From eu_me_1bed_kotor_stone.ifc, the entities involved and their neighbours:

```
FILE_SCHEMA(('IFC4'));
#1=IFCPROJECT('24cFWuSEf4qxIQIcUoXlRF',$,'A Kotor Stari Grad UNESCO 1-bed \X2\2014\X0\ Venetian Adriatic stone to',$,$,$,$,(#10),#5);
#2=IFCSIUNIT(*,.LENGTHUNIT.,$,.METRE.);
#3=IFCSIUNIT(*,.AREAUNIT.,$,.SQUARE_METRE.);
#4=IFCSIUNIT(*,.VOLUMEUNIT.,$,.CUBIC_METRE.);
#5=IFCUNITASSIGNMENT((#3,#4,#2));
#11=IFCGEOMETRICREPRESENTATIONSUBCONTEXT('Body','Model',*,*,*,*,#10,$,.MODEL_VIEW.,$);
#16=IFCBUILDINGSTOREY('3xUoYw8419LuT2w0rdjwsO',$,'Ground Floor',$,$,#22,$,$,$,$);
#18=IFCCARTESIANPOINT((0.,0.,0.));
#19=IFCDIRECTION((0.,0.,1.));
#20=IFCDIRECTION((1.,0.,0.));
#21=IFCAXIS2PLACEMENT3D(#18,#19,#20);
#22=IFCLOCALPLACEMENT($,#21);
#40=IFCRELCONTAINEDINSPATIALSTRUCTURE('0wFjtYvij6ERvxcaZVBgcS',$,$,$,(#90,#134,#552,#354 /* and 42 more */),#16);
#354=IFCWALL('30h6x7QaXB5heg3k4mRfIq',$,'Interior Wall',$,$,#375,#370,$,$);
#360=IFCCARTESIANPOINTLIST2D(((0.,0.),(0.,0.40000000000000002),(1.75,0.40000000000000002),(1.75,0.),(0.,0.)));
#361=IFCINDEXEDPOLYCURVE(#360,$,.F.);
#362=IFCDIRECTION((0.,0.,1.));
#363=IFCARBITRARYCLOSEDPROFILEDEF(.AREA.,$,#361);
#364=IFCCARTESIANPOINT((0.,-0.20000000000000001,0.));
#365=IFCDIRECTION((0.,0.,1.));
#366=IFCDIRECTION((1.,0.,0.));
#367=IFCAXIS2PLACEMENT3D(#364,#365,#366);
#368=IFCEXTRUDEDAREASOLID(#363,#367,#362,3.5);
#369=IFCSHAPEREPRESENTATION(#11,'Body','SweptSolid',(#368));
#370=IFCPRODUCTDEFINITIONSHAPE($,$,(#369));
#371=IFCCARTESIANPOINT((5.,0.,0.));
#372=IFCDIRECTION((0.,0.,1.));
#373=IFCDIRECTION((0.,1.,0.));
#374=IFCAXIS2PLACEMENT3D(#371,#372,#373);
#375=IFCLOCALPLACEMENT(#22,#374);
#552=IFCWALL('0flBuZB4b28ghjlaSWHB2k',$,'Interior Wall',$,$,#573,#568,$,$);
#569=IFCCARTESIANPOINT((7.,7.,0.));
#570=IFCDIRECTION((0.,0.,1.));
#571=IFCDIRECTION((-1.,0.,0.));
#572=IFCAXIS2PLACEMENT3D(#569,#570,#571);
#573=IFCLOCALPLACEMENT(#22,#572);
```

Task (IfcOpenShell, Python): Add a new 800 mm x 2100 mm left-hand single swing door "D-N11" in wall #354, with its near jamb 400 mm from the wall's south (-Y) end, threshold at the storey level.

```python
import numpy as np
import ifcopenshell
import ifcopenshell.api.feature
import ifcopenshell.api.geometry
import ifcopenshell.api.root
import ifcopenshell.api.spatial
import ifcopenshell.geom
import ifcopenshell.util.element
import ifcopenshell.util.placement
import ifcopenshell.util.representation
import ifcopenshell.util.shape
import ifcopenshell.util.unit

model = ifcopenshell.open("eu_me_1bed_kotor_stone.ifc")
unit_scale = ifcopenshell.util.unit.calculate_unit_scale(model)
settings = ifcopenshell.geom.settings()


def volume(element):
    """Net volume in cubic metres, openings subtracted."""
    shape = ifcopenshell.geom.create_shape(settings, element)
    return ifcopenshell.util.shape.get_volume(shape.geometry)


wall = model.by_id(354)
storey = ifcopenshell.util.element.get_container(wall, ifc_class="IfcBuildingStorey")
context = ifcopenshell.util.representation.get_context(model, "Model", "Body", "MODEL_VIEW")
before = volume(wall)

width, height, from_end, sill = 0.8, 2.1, 0.4, 0.0  # metres

# The wall runs along its own X axis, and the end named is its -X end.
wall_shape = ifcopenshell.geom.create_shape(settings, wall)
x, y, z = ifcopenshell.util.shape.get_vertices(wall_shape.geometry).T
start = x.min() + from_end
face, thickness = float(y.min()), float(y.max() - y.min())
wall_matrix = ifcopenshell.util.placement.get_local_placement(wall.ObjectPlacement)
level = ifcopenshell.util.placement.get_local_placement(storey.ObjectPlacement)[2, 3]


def in_wall(x, y):
    """Placement at x, y metres in the wall's axes, at sill height."""
    matrix = wall_matrix.copy()
    matrix[:, 3] = wall_matrix @ np.array([x / unit_scale, y / unit_scale, 0.0, 1.0])
    matrix[2, 3] = level + sill / unit_scale
    return matrix


# Opening: a box that overshoots both wall faces by 50 mm.
opening = ifcopenshell.api.root.create_entity(model, ifc_class="IfcOpeningElement", predefined_type="OPENING")
box = ifcopenshell.api.geometry.add_wall_representation(
    model, context=context, length=width, height=height, thickness=thickness + 0.1
)
ifcopenshell.api.geometry.assign_representation(model, product=opening, representation=box)
ifcopenshell.api.geometry.edit_object_placement(model, product=opening, matrix=in_wall(start, face - 0.05), is_si=False)
ifcopenshell.api.feature.add_feature(model, feature=opening, element=wall)

door = ifcopenshell.api.root.create_entity(model, ifc_class="IfcDoor", name="D-N11", predefined_type="DOOR")
door.OverallWidth, door.OverallHeight = width / unit_scale, height / unit_scale
door.OperationType = "SINGLE_SWING_LEFT"
body = ifcopenshell.api.geometry.add_door_representation(
    model,
    context=context,
    overall_width=door.OverallWidth,
    overall_height=door.OverallHeight,
    operation_type="SINGLE_SWING_LEFT",
    lining_properties={"LiningDepth": thickness / unit_scale, "ThresholdDepth": thickness / unit_scale},
)
ifcopenshell.api.geometry.assign_representation(model, product=door, representation=body)
ifcopenshell.api.spatial.assign_container(model, products=[door], relating_structure=storey)
ifcopenshell.api.feature.add_filling(model, opening=opening, element=door)

# The lining spans the wall, so the door starts at the wall face.
ifcopenshell.api.geometry.edit_object_placement(model, product=door, matrix=in_wall(start, face), is_si=False)

after = volume(wall)

print(f"wall volume {before:.3f} -> {after:.3f} m3")

model.write("eu_me_1bed_kotor_stone_updated.ifc")
```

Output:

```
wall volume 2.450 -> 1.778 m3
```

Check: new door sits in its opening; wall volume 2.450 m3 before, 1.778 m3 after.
